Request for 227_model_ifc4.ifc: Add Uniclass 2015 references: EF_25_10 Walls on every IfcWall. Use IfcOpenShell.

First a look at what the model holds.

```python
import ifcopenshell

model = ifcopenshell.open("227_model_ifc4.ifc")
print(model.schema)
print("classifications:", [c.Name for c in model.by_type("IfcClassification")])
for ifc_class in ("IfcDoor", "IfcRoof", "IfcStair", "IfcWall", "IfcWindow"):
    print(ifc_class, len(model.by_type(ifc_class)))
```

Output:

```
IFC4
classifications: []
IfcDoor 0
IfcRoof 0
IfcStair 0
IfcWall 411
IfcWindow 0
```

```python
import ifcopenshell
import ifcopenshell.api.classification

model = ifcopenshell.open("227_model_ifc4.ifc")

system = ifcopenshell.api.classification.add_classification(model, classification="Uniclass 2015")

codes = {
    "IfcWall": ("EF_25_10", "Walls"),
}
for ifc_class, (code, name) in codes.items():
    products = model.by_type(ifc_class)
    ifcopenshell.api.classification.add_reference(
        model, products=products, classification=system, identification=code, name=name
    )
    print(code, len(products))

model.write("227_model_ifc4_rev.ifc")
```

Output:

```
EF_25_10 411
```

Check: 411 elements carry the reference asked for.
